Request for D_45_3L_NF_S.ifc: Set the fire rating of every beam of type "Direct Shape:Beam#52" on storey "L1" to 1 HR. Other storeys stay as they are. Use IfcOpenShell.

First a look at what the model holds.

```python
import ifcopenshell
import ifcopenshell.util.element

model = ifcopenshell.open("D_45_3L_NF_S.ifc")
print(model.schema)
storey = next(s for s in model.by_type("IfcBuildingStorey") if s.Name == "L1")
beams = [e for e in ifcopenshell.util.element.get_decomposition(storey) if e.is_a("IfcBeam")]
seen = {}
for e in beams:
    element_type = ifcopenshell.util.element.get_type(e)
    key = (element_type.Name if element_type != e and element_type else None, ifcopenshell.util.element.get_pset(e, "Pset_BeamCommon", "FireRating"))
    seen[key] = seen.get(key, 0) + 1
for (name, value), count in sorted(seen.items(), key=str):
    print(count, "x", name, "|", value)
```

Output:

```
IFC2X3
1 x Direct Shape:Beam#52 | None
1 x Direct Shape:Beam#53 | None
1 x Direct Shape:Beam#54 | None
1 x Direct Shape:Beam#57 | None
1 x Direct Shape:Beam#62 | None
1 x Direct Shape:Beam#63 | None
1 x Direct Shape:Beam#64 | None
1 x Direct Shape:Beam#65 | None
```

```python
import ifcopenshell
import ifcopenshell.api.pset
import ifcopenshell.util.element

model = ifcopenshell.open("D_45_3L_NF_S.ifc")

storey = next(s for s in model.by_type("IfcBuildingStorey") if s.Name == "L1")
beams = [e for e in ifcopenshell.util.element.get_decomposition(storey) if e.is_a("IfcBeam")]

count = 0
for e in beams:
    element_type = ifcopenshell.util.element.get_type(e)
    if element_type in (None, e) or element_type.Name != "Direct Shape:Beam#52":
        continue
    # add_pset returns the element's existing set when there is one.
    pset = ifcopenshell.api.pset.add_pset(model, product=e, name="Pset_BeamCommon")
    ifcopenshell.api.pset.edit_pset(model, pset=pset, properties={"FireRating": "1 HR"})
    count += 1

print(count, "beams updated")

model.write("D_45_3L_NF_S_rev.ifc")
```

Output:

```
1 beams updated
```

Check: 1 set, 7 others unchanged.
